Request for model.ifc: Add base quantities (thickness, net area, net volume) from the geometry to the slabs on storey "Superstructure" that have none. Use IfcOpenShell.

First a look at what the model holds.

```python
import ifcopenshell
import ifcopenshell.util.element
import ifcopenshell.util.unit

model = ifcopenshell.open("model.ifc")
print(model.schema)
for unit_type in ("LENGTHUNIT", "AREAUNIT", "VOLUMEUNIT"):
    print(unit_type, ifcopenshell.util.unit.calculate_unit_scale(model, unit_type))
storey = next(s for s in model.by_type("IfcBuildingStorey") if s.Name == "Superstructure")
slabs = [e for e in ifcopenshell.util.element.get_decomposition(storey) if e.is_a("IfcSlab")]
for e in sorted(slabs, key=lambda e: e.id()):
    print(e.id(), e.is_a(), e.Name, list(ifcopenshell.util.element.get_psets(e, qtos_only=True)), sep=" | ")
```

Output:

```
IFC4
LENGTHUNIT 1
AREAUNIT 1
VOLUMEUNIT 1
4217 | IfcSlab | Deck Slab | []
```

```python
import ifcopenshell
import ifcopenshell.api.pset
import ifcopenshell.geom
import ifcopenshell.util.element
import ifcopenshell.util.shape
import ifcopenshell.util.unit

model = ifcopenshell.open("model.ifc")
unit_scale = ifcopenshell.util.unit.calculate_unit_scale(model)
area_scale = ifcopenshell.util.unit.calculate_unit_scale(model, "AREAUNIT")
volume_scale = ifcopenshell.util.unit.calculate_unit_scale(model, "VOLUMEUNIT")
settings = ifcopenshell.geom.settings()

storey = next(s for s in model.by_type("IfcBuildingStorey") if s.Name == "Superstructure")
slabs = [e for e in ifcopenshell.util.element.get_decomposition(storey) if e.is_a("IfcSlab")]

for e in sorted(slabs, key=lambda e: e.id()):
    if ifcopenshell.util.element.get_psets(e, qtos_only=True, should_inherit=False):
        continue
    # Geometry comes back in metres, in the element's own axes.
    shape = ifcopenshell.geom.create_shape(settings, e)
    values = {
        "Width": ifcopenshell.util.shape.get_z(shape.geometry) / unit_scale,
        "NetArea": ifcopenshell.util.shape.get_footprint_area(shape.geometry) / area_scale,
        "NetVolume": ifcopenshell.util.shape.get_volume(shape.geometry) / volume_scale,
    }
    qto = ifcopenshell.api.pset.add_qto(model, product=e, name="Qto_SlabBaseQuantities")
    ifcopenshell.api.pset.edit_qto(model, qto=qto, properties=values)
    print(e.id(), {k: round(v, 3) for k, v in values.items()})

model.write("model_v2.ifc")
```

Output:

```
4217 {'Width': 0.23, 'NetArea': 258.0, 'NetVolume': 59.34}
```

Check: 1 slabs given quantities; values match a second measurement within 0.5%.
